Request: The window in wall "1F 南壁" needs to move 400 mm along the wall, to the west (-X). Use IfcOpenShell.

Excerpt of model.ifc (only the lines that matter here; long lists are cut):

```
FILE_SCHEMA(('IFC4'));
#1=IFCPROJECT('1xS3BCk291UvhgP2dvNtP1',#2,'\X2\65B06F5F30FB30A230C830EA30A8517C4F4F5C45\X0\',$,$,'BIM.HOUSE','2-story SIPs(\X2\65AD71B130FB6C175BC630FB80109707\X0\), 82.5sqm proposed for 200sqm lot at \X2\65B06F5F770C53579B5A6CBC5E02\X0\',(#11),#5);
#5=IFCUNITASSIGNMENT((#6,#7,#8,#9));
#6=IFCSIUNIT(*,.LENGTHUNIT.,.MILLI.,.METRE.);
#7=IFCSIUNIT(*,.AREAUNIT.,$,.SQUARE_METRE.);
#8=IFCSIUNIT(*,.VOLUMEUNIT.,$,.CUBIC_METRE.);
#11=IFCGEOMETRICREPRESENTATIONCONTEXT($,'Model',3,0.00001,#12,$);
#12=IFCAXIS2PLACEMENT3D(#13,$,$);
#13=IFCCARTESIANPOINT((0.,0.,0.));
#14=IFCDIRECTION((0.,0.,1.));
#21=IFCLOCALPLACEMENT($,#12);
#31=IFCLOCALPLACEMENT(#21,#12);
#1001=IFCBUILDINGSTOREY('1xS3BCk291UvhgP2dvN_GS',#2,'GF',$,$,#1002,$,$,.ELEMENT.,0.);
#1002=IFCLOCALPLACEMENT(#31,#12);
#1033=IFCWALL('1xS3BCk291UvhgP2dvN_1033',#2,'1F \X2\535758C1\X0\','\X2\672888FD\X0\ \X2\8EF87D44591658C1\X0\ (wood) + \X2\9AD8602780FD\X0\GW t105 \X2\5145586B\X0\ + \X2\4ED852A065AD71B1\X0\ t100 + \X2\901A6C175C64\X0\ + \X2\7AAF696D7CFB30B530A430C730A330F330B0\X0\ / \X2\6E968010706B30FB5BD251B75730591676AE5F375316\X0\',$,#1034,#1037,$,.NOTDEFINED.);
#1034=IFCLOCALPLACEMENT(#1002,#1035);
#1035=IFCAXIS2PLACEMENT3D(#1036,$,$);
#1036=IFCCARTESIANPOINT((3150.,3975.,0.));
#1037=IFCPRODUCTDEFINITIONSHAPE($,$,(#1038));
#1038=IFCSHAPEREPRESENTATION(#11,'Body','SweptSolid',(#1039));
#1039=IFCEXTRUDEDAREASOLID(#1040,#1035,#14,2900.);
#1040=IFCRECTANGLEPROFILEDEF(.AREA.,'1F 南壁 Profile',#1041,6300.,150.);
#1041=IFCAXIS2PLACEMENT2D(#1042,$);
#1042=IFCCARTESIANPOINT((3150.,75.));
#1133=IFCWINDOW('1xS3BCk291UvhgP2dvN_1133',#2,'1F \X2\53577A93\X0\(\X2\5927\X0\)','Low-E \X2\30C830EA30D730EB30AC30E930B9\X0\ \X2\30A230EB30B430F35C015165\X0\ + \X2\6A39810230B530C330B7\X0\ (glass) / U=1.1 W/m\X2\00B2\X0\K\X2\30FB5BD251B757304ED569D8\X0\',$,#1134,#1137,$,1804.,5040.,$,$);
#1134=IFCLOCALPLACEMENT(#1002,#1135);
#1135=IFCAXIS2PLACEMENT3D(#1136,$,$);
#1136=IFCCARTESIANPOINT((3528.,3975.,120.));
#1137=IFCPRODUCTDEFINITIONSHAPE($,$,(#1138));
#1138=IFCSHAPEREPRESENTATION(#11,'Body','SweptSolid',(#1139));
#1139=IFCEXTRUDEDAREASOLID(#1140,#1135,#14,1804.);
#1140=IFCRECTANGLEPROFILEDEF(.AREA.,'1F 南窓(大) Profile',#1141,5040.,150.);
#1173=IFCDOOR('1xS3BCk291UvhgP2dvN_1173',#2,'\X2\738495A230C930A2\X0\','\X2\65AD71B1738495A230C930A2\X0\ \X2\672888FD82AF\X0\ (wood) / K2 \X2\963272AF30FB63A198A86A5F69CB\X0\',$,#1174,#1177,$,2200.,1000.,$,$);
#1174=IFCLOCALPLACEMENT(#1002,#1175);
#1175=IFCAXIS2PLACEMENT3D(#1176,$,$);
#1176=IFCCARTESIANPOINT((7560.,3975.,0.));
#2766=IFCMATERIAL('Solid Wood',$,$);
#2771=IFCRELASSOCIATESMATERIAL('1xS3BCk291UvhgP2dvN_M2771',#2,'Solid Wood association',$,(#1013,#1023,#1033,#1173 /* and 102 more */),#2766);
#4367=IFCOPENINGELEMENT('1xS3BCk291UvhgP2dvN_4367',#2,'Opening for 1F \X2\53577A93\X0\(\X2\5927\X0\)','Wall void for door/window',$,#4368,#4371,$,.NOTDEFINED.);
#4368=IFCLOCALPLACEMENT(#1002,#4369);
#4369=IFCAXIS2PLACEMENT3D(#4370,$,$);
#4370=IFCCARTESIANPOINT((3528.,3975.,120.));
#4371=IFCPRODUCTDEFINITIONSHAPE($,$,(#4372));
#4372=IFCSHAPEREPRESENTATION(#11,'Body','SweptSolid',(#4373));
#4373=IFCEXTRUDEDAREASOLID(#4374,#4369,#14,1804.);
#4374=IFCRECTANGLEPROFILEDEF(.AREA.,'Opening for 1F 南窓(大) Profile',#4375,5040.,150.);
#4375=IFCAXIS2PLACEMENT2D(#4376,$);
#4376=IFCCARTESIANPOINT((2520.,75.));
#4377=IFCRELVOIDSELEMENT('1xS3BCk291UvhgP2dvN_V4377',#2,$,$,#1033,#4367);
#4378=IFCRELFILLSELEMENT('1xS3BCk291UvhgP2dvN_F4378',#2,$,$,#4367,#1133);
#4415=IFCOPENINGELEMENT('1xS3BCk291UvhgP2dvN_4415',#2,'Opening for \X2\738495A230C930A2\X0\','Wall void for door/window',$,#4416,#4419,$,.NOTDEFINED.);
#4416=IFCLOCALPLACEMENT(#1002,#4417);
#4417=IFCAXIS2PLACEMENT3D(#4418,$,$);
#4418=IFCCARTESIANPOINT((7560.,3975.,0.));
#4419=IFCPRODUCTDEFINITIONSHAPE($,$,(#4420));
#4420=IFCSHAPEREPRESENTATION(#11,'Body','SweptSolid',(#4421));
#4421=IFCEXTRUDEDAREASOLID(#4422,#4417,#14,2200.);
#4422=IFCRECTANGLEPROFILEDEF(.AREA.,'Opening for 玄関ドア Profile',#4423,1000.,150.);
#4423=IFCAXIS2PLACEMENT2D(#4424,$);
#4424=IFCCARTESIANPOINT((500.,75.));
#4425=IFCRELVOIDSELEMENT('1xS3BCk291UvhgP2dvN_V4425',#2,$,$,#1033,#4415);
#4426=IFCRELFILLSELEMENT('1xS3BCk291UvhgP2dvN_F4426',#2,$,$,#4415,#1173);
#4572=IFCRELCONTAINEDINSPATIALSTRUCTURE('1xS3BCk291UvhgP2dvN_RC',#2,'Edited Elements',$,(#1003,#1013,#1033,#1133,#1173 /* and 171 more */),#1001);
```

```python
import ifcopenshell
import ifcopenshell.api.geometry
import ifcopenshell.util.placement

model = ifcopenshell.open("model.ifc")

window = model.by_guid("1xS3BCk291UvhgP2dvN_1133")
opening = window.FillsVoids[0].RelatingOpeningElement
wall = opening.VoidsElements[0].RelatingBuildingElement

wall_matrix = ifcopenshell.util.placement.get_local_placement(wall.ObjectPlacement)
shift = wall_matrix[:3, 0] * -400.0
before = ifcopenshell.util.placement.get_local_placement(window.ObjectPlacement)[:3, 3].copy()

# The window is not placed relative to its opening, so move both.
for product in (opening, window):
    matrix = ifcopenshell.util.placement.get_local_placement(product.ObjectPlacement)
    matrix[:3, 3] += shift
    ifcopenshell.api.geometry.edit_object_placement(model, product=product, matrix=matrix, is_si=False)

after = ifcopenshell.util.placement.get_local_placement(window.ObjectPlacement)[:3, 3]
print("window moved by", (after - before).round(3) + 0.0)

model.write("model_rev.ifc")
```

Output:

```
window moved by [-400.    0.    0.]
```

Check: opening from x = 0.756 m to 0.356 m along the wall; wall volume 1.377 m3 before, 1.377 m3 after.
